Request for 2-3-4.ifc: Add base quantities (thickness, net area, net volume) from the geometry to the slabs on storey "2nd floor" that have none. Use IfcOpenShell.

First a look at what the model holds.

```python
import ifcopenshell
import ifcopenshell.util.element
import ifcopenshell.util.unit

model = ifcopenshell.open("2-3-4.ifc")
print(model.schema)
for unit_type in ("LENGTHUNIT", "AREAUNIT", "VOLUMEUNIT"):
    print(unit_type, ifcopenshell.util.unit.calculate_unit_scale(model, unit_type))
storey = next(s for s in model.by_type("IfcBuildingStorey") if s.Name == "2nd floor")
slabs = [e for e in ifcopenshell.util.element.get_decomposition(storey) if e.is_a("IfcSlab")]
for e in sorted(slabs, key=lambda e: e.id()):
    print(e.id(), e.is_a(), e.Name, list(ifcopenshell.util.element.get_psets(e, qtos_only=True)), sep=" | ")
```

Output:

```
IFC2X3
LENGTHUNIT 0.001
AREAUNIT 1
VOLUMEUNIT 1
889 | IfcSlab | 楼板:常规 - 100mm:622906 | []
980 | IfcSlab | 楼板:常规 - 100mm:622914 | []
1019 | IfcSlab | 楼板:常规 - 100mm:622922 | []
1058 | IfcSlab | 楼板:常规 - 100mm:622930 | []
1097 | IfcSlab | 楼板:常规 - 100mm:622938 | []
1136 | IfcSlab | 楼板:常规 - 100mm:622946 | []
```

```python
import ifcopenshell
import ifcopenshell.api.pset
import ifcopenshell.geom
import ifcopenshell.util.element
import ifcopenshell.util.shape
import ifcopenshell.util.unit

model = ifcopenshell.open("2-3-4.ifc")
unit_scale = ifcopenshell.util.unit.calculate_unit_scale(model)
area_scale = ifcopenshell.util.unit.calculate_unit_scale(model, "AREAUNIT")
volume_scale = ifcopenshell.util.unit.calculate_unit_scale(model, "VOLUMEUNIT")
settings = ifcopenshell.geom.settings()

storey = next(s for s in model.by_type("IfcBuildingStorey") if s.Name == "2nd floor")
slabs = [e for e in ifcopenshell.util.element.get_decomposition(storey) if e.is_a("IfcSlab")]

for e in sorted(slabs, key=lambda e: e.id()):
    if ifcopenshell.util.element.get_psets(e, qtos_only=True, should_inherit=False):
        continue
    # Geometry comes back in metres, in the element's own axes.
    shape = ifcopenshell.geom.create_shape(settings, e)
    values = {
        "Width": ifcopenshell.util.shape.get_z(shape.geometry) / unit_scale,
        "NetArea": ifcopenshell.util.shape.get_footprint_area(shape.geometry) / area_scale,
        "NetVolume": ifcopenshell.util.shape.get_volume(shape.geometry) / volume_scale,
    }
    qto = ifcopenshell.api.pset.add_qto(model, product=e, name="BaseQuantities")
    ifcopenshell.api.pset.edit_qto(model, qto=qto, properties=values)
    print(e.id(), {k: round(v, 3) for k, v in values.items()})

model.write("2-3-4_rev.ifc")
```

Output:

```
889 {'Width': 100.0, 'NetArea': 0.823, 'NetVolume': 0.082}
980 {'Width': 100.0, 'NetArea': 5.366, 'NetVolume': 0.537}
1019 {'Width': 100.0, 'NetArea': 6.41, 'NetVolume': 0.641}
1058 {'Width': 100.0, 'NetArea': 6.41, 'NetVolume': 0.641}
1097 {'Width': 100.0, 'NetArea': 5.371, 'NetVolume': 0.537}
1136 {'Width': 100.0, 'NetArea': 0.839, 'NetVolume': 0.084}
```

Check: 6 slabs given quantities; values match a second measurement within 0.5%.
